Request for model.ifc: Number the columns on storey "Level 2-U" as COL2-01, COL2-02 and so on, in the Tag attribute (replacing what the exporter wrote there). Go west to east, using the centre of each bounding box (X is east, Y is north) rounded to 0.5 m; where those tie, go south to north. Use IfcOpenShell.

First a look at what the model holds.

```python
import ifcopenshell
import ifcopenshell.util.element
import ifcopenshell.util.placement

model = ifcopenshell.open("model.ifc")
print(model.schema)
storey = next(s for s in model.by_type("IfcBuildingStorey") if s.Name == "Level 2-U")
columns = [e for e in ifcopenshell.util.element.get_decomposition(storey) if e.is_a("IfcColumn")]
for e in sorted(columns, key=lambda e: e.id()):
    origin = ifcopenshell.util.placement.get_local_placement(e.ObjectPlacement)[:3, 3]
    print(e.id(), e.Tag, e.Name, origin.round(2) + 0.0, sep=" | ")
```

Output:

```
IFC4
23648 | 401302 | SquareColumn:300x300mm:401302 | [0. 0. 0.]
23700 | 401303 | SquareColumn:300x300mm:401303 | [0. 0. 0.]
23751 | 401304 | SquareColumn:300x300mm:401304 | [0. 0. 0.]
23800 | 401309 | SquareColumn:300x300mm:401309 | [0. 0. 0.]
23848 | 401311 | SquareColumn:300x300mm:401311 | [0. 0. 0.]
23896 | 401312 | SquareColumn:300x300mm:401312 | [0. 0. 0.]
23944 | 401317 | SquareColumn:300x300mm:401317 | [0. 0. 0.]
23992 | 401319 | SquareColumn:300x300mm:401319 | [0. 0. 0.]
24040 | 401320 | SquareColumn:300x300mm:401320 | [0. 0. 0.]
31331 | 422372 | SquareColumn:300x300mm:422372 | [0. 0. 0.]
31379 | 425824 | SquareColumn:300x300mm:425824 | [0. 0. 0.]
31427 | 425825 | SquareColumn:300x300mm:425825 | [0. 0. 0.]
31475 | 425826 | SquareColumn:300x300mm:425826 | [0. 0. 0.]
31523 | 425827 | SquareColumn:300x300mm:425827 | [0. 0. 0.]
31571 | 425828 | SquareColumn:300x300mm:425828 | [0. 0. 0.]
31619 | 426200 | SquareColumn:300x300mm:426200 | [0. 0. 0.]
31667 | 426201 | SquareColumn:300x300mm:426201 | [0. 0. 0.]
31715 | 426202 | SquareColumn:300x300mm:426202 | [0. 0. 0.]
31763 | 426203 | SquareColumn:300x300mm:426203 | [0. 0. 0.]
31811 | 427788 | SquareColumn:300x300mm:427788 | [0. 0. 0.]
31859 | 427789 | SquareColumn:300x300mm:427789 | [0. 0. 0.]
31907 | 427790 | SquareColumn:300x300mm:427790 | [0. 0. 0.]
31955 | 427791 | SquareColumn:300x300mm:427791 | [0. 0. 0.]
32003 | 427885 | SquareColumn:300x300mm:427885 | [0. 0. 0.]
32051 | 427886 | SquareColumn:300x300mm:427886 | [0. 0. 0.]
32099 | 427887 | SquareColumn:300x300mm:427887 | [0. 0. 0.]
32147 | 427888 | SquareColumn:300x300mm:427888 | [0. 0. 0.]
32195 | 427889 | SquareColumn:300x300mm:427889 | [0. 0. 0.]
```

```python
import ifcopenshell
import ifcopenshell.geom
import ifcopenshell.util.element
import ifcopenshell.util.shape

model = ifcopenshell.open("model.ifc")
settings = ifcopenshell.geom.settings()
settings.set("use-world-coords", True)


def centre(element):
    shape = ifcopenshell.geom.create_shape(settings, element)
    return ifcopenshell.util.shape.get_bbox_centroid(shape.geometry)


storey = next(s for s in model.by_type("IfcBuildingStorey") if s.Name == "Level 2-U")
columns = [e for e in ifcopenshell.util.element.get_decomposition(storey) if e.is_a("IfcColumn")]

# Insertion points can sit at a corner or the storey origin, so sort by the geometry (in metres).
centres = {e: centre(e) for e in columns}
columns.sort(key=lambda e: (round(centres[e][0] / 0.5), centres[e][1]))

for i, e in enumerate(columns, start=1):
    number = f"COL2-{i:02d}"
    e.Tag = number
    print(e.id(), number)

model.write("model_updated.ifc")
```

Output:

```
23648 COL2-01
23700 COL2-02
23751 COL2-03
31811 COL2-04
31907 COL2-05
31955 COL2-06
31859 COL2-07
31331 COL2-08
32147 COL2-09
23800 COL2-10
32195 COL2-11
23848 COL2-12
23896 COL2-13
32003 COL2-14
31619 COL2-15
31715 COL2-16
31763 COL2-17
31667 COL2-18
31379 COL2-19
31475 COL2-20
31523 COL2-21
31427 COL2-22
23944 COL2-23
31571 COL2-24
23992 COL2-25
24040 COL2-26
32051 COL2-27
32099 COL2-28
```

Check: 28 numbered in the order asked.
